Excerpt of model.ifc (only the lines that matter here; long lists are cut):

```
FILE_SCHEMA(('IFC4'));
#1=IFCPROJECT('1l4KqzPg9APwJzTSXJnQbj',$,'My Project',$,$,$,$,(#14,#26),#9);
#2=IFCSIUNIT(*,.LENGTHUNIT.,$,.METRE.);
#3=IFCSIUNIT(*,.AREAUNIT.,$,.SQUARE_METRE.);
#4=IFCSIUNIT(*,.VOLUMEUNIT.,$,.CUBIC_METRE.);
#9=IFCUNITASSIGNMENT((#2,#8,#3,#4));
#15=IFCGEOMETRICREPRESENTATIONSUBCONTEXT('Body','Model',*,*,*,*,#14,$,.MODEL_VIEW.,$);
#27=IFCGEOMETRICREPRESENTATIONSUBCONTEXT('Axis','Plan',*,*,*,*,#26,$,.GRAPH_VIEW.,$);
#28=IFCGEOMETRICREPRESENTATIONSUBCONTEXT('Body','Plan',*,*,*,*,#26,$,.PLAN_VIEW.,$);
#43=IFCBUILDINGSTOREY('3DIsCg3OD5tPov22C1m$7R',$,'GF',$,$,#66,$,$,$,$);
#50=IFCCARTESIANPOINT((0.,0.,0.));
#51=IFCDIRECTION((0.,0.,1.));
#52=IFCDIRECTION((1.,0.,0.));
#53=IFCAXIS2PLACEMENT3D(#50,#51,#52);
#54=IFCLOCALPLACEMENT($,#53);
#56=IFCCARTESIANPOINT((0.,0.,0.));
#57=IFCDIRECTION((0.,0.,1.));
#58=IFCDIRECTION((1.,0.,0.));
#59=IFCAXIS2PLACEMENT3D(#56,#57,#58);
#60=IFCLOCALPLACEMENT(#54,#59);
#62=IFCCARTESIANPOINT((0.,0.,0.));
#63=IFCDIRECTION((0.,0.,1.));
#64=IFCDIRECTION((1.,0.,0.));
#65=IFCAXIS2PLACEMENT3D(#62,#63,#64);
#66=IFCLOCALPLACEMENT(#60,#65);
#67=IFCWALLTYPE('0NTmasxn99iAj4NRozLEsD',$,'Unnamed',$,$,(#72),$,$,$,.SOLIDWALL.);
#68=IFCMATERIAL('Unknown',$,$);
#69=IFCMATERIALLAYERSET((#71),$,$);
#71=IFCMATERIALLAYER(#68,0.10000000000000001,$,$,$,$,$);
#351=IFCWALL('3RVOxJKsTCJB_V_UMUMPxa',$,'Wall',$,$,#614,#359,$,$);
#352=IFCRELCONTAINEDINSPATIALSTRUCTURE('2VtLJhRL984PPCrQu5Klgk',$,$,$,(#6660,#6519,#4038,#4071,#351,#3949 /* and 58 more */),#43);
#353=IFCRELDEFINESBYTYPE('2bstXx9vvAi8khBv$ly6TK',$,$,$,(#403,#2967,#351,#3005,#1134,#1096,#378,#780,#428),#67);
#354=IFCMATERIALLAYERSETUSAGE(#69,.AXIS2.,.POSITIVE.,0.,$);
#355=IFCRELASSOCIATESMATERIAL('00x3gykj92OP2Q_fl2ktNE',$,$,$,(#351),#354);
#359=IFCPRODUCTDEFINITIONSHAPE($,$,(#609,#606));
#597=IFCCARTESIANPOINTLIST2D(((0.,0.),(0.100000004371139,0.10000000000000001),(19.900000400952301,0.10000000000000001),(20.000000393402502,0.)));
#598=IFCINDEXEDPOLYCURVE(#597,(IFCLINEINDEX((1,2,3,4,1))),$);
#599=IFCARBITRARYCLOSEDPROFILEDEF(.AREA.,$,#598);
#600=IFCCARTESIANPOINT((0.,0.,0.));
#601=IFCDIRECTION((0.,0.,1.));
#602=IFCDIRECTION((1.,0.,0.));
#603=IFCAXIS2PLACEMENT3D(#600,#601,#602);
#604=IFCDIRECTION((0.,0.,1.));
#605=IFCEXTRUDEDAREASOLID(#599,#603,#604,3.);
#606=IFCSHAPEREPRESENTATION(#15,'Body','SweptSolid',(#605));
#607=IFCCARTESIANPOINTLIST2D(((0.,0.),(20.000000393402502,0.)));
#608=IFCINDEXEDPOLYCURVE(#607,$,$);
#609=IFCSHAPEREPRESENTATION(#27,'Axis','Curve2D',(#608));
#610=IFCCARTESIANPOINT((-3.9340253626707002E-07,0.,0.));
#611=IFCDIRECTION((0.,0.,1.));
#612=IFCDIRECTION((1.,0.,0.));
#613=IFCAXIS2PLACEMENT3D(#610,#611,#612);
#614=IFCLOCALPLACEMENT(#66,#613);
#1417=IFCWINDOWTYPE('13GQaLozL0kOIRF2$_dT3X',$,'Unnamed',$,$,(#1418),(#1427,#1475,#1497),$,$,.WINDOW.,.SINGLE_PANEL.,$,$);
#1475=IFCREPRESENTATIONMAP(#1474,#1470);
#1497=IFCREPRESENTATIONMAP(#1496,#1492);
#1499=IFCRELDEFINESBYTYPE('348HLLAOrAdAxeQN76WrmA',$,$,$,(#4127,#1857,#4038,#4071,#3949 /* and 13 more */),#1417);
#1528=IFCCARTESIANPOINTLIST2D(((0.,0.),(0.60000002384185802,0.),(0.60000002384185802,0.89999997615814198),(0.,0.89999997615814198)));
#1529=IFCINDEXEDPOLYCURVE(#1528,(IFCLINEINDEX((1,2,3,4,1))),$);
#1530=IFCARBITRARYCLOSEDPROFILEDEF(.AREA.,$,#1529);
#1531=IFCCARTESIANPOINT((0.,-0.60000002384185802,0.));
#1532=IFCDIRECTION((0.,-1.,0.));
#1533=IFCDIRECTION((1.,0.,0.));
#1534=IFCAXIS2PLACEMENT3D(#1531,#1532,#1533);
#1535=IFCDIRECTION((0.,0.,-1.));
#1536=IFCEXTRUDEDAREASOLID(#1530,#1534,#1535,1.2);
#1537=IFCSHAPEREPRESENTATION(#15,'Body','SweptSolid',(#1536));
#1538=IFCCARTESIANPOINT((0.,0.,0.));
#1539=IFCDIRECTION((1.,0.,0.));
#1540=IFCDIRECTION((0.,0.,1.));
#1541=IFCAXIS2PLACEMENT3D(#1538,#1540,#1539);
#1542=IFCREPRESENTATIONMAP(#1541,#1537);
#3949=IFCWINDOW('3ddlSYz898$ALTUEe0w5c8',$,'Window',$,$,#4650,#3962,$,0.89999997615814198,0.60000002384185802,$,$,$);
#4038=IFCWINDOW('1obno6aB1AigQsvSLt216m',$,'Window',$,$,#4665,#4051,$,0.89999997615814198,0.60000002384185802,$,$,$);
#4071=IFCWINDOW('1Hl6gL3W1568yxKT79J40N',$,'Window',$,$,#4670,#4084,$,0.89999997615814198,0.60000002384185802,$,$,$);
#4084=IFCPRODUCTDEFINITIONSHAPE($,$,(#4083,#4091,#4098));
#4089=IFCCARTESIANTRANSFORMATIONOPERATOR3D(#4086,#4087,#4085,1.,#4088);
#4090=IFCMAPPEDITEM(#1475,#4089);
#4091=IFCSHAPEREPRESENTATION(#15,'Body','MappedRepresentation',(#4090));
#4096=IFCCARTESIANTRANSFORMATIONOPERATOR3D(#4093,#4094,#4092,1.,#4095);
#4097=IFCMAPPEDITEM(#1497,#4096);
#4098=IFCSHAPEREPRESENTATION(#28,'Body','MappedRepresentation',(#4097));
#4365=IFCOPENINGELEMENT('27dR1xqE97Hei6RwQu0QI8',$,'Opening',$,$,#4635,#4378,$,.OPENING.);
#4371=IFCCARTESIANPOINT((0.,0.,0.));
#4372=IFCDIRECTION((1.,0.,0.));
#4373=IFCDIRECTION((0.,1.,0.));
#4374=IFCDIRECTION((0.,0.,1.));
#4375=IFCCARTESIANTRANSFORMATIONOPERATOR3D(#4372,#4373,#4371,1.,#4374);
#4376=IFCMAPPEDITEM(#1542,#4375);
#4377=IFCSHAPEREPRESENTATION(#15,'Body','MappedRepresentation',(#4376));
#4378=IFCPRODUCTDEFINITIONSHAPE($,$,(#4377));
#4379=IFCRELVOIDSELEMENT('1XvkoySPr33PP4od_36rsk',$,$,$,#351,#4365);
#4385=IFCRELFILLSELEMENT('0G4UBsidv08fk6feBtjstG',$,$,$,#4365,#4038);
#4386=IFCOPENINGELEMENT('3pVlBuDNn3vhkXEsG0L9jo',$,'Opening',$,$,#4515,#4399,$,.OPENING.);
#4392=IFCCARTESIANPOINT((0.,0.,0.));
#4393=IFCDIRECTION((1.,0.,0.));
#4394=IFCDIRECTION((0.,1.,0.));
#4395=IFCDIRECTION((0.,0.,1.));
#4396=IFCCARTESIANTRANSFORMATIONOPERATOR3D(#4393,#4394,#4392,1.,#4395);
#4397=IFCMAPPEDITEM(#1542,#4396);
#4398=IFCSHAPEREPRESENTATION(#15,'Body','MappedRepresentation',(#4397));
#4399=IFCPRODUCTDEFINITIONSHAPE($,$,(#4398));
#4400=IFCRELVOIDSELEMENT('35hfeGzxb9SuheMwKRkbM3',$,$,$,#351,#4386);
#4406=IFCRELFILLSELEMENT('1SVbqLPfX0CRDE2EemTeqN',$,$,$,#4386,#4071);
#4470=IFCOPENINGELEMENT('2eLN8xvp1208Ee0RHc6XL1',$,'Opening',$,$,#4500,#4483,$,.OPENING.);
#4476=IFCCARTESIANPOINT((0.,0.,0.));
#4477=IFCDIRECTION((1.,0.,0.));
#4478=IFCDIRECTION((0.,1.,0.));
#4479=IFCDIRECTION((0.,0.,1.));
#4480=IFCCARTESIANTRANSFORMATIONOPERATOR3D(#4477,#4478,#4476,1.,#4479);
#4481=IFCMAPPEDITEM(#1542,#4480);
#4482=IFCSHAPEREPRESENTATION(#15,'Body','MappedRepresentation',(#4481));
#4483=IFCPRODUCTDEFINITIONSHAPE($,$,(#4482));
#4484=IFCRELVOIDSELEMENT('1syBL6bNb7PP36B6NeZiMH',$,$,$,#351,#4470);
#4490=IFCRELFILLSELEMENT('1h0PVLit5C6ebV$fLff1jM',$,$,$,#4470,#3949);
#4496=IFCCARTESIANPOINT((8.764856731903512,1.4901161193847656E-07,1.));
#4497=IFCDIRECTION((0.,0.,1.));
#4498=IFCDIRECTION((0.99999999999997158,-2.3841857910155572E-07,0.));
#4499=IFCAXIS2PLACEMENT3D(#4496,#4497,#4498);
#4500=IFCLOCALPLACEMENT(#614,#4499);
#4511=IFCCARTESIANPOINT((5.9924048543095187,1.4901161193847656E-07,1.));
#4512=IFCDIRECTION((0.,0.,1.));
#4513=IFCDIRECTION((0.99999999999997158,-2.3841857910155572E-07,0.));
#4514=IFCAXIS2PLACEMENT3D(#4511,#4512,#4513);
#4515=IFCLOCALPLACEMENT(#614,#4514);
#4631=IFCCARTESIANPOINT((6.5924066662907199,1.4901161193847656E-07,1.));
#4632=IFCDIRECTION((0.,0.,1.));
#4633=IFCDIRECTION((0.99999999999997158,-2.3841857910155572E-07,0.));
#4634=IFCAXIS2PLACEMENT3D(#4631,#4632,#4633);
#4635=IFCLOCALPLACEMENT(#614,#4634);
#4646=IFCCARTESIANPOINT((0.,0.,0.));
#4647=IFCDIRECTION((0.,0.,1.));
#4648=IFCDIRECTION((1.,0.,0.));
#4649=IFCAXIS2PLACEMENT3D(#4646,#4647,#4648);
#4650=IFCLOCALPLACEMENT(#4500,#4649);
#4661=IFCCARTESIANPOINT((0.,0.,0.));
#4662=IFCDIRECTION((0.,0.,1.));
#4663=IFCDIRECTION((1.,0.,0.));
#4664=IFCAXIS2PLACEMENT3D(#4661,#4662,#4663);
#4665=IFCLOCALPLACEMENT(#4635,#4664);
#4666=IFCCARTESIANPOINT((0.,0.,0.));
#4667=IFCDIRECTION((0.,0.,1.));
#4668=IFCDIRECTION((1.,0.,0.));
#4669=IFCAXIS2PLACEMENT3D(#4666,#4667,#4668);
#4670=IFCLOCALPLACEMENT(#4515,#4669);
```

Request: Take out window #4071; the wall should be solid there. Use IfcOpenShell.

```python
import ifcopenshell
import ifcopenshell.api.feature
import ifcopenshell.api.root
import ifcopenshell.geom
import ifcopenshell.util.shape

model = ifcopenshell.open("model.ifc")
settings = ifcopenshell.geom.settings()


def volume(element):
    """Net volume in cubic metres, openings subtracted."""
    shape = ifcopenshell.geom.create_shape(settings, element)
    return ifcopenshell.util.shape.get_volume(shape.geometry)


window = model.by_guid("1Hl6gL3W1568yxKT79J40N")
opening = window.FillsVoids[0].RelatingOpeningElement
wall = opening.VoidsElements[0].RelatingBuildingElement
before = volume(wall)

ifcopenshell.api.root.remove_product(model, product=window)
ifcopenshell.api.feature.remove_feature(model, feature=opening)

after = volume(wall)

print(f"wall volume {before:.3f} -> {after:.3f} m3")

model.write("model_rev.ifc")
```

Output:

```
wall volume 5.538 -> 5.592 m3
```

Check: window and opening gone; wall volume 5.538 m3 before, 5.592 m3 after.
